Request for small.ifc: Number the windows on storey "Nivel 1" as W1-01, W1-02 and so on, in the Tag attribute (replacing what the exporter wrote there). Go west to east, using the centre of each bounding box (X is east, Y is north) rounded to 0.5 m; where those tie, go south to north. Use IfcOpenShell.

First a look at what the model holds.

```python
import ifcopenshell
import ifcopenshell.util.element
import ifcopenshell.util.placement

model = ifcopenshell.open("small.ifc")
print(model.schema)
storey = next(s for s in model.by_type("IfcBuildingStorey") if s.Name == "Nivel 1")
windows = [e for e in ifcopenshell.util.element.get_decomposition(storey) if e.is_a("IfcWindow")]
for e in sorted(windows, key=lambda e: e.id()):
    origin = ifcopenshell.util.placement.get_local_placement(e.ObjectPlacement)[:3, 3]
    print(e.id(), e.Tag, e.Name, origin.round(2) + 0.0, sep=" | ")
```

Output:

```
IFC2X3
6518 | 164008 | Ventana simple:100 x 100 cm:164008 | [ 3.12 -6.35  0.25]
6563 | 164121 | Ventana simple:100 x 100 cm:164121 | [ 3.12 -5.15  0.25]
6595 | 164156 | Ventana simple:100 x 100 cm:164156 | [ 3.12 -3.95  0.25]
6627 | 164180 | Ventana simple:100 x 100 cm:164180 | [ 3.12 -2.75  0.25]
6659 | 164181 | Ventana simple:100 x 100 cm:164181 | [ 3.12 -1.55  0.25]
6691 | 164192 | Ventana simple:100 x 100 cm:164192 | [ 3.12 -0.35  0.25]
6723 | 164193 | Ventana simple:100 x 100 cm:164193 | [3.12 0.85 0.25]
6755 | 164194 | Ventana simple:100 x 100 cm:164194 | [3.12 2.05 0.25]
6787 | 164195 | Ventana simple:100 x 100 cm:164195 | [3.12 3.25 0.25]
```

```python
import ifcopenshell
import ifcopenshell.geom
import ifcopenshell.util.element
import ifcopenshell.util.shape

model = ifcopenshell.open("small.ifc")
settings = ifcopenshell.geom.settings()
settings.set("use-world-coords", True)


def centre(element):
    shape = ifcopenshell.geom.create_shape(settings, element)
    return ifcopenshell.util.shape.get_bbox_centroid(shape.geometry)


storey = next(s for s in model.by_type("IfcBuildingStorey") if s.Name == "Nivel 1")
windows = [e for e in ifcopenshell.util.element.get_decomposition(storey) if e.is_a("IfcWindow")]

# Insertion points can sit at a corner or the storey origin, so sort by the geometry (in metres).
centres = {e: centre(e) for e in windows}
windows.sort(key=lambda e: (round(centres[e][0] / 0.5), centres[e][1]))

for i, e in enumerate(windows, start=1):
    number = f"W1-{i:02d}"
    e.Tag = number
    print(e.id(), number)

model.write("small_edited.ifc")
```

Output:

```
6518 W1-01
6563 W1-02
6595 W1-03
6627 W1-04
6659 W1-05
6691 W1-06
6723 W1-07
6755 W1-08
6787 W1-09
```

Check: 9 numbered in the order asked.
